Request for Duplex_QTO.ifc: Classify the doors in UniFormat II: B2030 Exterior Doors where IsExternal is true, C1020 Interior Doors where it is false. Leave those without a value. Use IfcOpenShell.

First a look at what the model holds.

```python
import ifcopenshell
import ifcopenshell.util.element

model = ifcopenshell.open("Duplex_QTO.ifc")
print(model.schema)
print("classifications:", [c.Name for c in model.by_type("IfcClassification")])
values = [ifcopenshell.util.element.get_pset(e, "Pset_DoorCommon", "IsExternal") for e in model.by_type("IfcDoor")]
for value in (True, False, None):
    print("IsExternal", value, values.count(value))
```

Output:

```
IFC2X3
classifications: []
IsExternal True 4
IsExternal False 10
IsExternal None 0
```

```python
import ifcopenshell
import ifcopenshell.api.classification
import ifcopenshell.util.element

model = ifcopenshell.open("Duplex_QTO.ifc")

# IFC2X3 requires Source and Edition and has no link from the project to the system.
system = model.create_entity("IfcClassification", Source="ASTM", Edition="E1557", Name="UniFormat II")

doors = model.by_type("IfcDoor")
external = {e: ifcopenshell.util.element.get_pset(e, "Pset_DoorCommon", "IsExternal") for e in doors}
for flag, code, name in ((True, "B2030", "Exterior Doors"), (False, "C1020", "Interior Doors")):
    products = [e for e in doors if external[e] is flag]
    ifcopenshell.api.classification.add_reference(
        model, products=products, classification=system, identification=code, name=name
    )
    print(code, len(products))

model.write("Duplex_QTO_rev.ifc")
```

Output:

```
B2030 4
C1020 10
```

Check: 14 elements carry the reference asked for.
